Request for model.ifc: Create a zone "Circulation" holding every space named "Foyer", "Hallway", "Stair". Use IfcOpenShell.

First a look at what the model holds.

```python
import ifcopenshell

model = ifcopenshell.open("model.ifc")
print(model.schema)
seen = {}
for space in model.by_type("IfcSpace"):
    seen[space.LongName] = seen.get(space.LongName, 0) + 1
for name, count in sorted(seen.items(), key=str):
    print(count, "x", name)
print("zones:", [z.Name for z in model.by_type("IfcZone")][:20])
```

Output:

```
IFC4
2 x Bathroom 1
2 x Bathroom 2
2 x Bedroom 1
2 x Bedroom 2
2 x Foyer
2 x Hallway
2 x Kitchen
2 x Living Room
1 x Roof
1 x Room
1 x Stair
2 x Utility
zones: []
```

```python
import ifcopenshell
import ifcopenshell.api.group
import ifcopenshell.api.root

model = ifcopenshell.open("model.ifc")

names = {"Foyer", "Hallway", "Stair"}
spaces = [s for s in model.by_type("IfcSpace") if s.LongName in names]

zone = ifcopenshell.api.root.create_entity(model, ifc_class="IfcZone", name="Circulation")
ifcopenshell.api.group.assign_group(model, products=spaces, group=zone)
print(len(spaces), "spaces in", zone.Name)

model.write("model_v2.ifc")
```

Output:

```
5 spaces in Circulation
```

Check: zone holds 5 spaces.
